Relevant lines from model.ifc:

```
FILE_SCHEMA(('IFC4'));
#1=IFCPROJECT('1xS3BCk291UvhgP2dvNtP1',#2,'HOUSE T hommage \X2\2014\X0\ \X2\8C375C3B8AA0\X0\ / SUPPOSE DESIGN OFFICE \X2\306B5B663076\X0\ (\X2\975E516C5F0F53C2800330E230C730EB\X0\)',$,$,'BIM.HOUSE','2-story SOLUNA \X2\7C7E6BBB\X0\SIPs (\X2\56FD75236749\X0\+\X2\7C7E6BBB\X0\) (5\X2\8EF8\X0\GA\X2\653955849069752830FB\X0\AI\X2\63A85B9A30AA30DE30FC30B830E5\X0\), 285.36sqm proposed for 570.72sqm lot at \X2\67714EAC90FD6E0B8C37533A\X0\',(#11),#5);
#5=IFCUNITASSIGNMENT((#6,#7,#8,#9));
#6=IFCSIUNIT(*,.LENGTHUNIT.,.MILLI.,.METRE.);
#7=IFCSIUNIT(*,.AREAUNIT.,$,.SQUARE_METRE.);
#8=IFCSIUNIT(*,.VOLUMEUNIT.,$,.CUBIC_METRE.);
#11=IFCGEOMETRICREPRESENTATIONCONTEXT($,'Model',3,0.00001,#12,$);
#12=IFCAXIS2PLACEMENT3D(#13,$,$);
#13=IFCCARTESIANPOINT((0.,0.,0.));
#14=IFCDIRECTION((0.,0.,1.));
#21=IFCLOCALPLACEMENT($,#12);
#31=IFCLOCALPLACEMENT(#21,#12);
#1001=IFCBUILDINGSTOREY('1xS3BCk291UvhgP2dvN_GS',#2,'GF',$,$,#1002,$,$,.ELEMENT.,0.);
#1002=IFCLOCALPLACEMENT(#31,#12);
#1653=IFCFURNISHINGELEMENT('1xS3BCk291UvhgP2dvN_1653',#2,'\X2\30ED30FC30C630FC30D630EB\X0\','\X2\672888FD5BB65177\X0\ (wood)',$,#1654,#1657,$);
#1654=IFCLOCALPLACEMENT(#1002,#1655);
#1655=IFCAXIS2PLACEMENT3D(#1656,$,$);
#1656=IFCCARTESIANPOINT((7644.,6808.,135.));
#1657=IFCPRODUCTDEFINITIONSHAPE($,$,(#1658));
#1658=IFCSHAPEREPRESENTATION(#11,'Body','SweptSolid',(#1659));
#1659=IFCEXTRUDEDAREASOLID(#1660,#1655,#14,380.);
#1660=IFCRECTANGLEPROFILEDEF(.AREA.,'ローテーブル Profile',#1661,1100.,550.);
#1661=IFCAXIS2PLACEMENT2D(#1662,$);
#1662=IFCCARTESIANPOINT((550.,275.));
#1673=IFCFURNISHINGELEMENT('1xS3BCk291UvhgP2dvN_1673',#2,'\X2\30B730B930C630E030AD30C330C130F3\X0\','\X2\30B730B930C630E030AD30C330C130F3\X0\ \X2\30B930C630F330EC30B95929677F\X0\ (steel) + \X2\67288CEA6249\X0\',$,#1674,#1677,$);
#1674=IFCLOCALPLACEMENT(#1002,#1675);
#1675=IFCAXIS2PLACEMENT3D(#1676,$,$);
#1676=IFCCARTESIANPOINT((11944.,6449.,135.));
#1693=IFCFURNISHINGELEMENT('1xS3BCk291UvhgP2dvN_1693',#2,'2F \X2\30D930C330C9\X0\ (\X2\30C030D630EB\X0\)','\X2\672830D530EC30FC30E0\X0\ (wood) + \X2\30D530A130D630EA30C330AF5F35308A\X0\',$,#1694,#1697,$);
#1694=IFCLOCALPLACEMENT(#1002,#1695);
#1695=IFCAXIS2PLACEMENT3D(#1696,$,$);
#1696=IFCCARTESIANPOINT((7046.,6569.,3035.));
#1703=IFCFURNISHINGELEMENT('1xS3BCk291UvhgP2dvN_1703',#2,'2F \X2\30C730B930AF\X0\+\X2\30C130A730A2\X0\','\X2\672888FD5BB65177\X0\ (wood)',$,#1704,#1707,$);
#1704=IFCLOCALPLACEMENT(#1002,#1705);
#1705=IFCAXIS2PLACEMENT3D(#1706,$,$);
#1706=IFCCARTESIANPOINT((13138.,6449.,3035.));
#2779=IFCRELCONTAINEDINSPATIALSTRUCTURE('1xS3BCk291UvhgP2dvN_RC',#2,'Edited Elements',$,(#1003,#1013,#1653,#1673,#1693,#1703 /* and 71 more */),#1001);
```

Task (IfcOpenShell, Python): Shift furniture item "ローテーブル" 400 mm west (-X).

```python
import ifcopenshell
import ifcopenshell.api.geometry
import ifcopenshell.util.placement
import ifcopenshell.util.unit

model = ifcopenshell.open("model.ifc")
unit_scale = ifcopenshell.util.unit.calculate_unit_scale(model)

item = model.by_id(1653)
matrix = ifcopenshell.util.placement.get_local_placement(item.ObjectPlacement)
matrix[0, 3] -= 0.4 / unit_scale
ifcopenshell.api.geometry.edit_object_placement(model, product=item, matrix=matrix, is_si=False)

print(ifcopenshell.util.placement.get_local_placement(item.ObjectPlacement).round(3) + 0.0)

model.write("model_rev.ifc")
```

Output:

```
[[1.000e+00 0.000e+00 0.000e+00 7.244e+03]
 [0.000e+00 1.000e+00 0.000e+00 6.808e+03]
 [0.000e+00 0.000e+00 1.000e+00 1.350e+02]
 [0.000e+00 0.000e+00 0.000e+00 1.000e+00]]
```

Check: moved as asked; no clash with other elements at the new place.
